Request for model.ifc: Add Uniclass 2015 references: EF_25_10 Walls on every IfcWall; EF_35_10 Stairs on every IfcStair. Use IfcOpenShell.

First a look at what the model holds.

```python
import ifcopenshell

model = ifcopenshell.open("model.ifc")
print(model.schema)
print("classifications:", [c.Name for c in model.by_type("IfcClassification")])
for ifc_class in ("IfcDoor", "IfcRoof", "IfcStair", "IfcWall", "IfcWindow"):
    print(ifc_class, len(model.by_type(ifc_class)))
```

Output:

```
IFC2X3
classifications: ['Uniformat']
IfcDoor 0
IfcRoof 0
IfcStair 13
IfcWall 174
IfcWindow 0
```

```python
import ifcopenshell
import ifcopenshell.api.classification

model = ifcopenshell.open("model.ifc")

# IFC2X3 requires Source and Edition and has no link from the project to the system.
system = model.create_entity("IfcClassification", Source="NBS", Edition="2015", Name="Uniclass 2015")

codes = {
    "IfcWall": ("EF_25_10", "Walls"),
    "IfcStair": ("EF_35_10", "Stairs"),
}
for ifc_class, (code, name) in codes.items():
    products = model.by_type(ifc_class)
    ifcopenshell.api.classification.add_reference(
        model, products=products, classification=system, identification=code, name=name
    )
    print(code, len(products))

model.write("model_v2.ifc")
```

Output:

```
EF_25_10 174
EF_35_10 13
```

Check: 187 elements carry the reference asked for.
